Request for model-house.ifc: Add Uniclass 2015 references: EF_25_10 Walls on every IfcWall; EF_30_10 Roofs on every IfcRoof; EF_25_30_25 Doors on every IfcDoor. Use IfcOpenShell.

First a look at what the model holds.

```python
import ifcopenshell

model = ifcopenshell.open("model-house.ifc")
print(model.schema)
print("classifications:", [c.Name for c in model.by_type("IfcClassification")])
for ifc_class in ("IfcDoor", "IfcRoof", "IfcStair", "IfcWall", "IfcWindow"):
    print(ifc_class, len(model.by_type(ifc_class)))
```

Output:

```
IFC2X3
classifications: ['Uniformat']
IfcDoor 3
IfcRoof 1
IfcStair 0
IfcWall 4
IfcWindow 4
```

```python
import ifcopenshell
import ifcopenshell.api.classification

model = ifcopenshell.open("model-house.ifc")

# IFC2X3 requires Source and Edition and has no link from the project to the system.
system = model.create_entity("IfcClassification", Source="NBS", Edition="2015", Name="Uniclass 2015")

codes = {
    "IfcWall": ("EF_25_10", "Walls"),
    "IfcRoof": ("EF_30_10", "Roofs"),
    "IfcDoor": ("EF_25_30_25", "Doors"),
}
for ifc_class, (code, name) in codes.items():
    products = model.by_type(ifc_class)
    ifcopenshell.api.classification.add_reference(
        model, products=products, classification=system, identification=code, name=name
    )
    print(code, len(products))

model.write("model-house-out.ifc")
```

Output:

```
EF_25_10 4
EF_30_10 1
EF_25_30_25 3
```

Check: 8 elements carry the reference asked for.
